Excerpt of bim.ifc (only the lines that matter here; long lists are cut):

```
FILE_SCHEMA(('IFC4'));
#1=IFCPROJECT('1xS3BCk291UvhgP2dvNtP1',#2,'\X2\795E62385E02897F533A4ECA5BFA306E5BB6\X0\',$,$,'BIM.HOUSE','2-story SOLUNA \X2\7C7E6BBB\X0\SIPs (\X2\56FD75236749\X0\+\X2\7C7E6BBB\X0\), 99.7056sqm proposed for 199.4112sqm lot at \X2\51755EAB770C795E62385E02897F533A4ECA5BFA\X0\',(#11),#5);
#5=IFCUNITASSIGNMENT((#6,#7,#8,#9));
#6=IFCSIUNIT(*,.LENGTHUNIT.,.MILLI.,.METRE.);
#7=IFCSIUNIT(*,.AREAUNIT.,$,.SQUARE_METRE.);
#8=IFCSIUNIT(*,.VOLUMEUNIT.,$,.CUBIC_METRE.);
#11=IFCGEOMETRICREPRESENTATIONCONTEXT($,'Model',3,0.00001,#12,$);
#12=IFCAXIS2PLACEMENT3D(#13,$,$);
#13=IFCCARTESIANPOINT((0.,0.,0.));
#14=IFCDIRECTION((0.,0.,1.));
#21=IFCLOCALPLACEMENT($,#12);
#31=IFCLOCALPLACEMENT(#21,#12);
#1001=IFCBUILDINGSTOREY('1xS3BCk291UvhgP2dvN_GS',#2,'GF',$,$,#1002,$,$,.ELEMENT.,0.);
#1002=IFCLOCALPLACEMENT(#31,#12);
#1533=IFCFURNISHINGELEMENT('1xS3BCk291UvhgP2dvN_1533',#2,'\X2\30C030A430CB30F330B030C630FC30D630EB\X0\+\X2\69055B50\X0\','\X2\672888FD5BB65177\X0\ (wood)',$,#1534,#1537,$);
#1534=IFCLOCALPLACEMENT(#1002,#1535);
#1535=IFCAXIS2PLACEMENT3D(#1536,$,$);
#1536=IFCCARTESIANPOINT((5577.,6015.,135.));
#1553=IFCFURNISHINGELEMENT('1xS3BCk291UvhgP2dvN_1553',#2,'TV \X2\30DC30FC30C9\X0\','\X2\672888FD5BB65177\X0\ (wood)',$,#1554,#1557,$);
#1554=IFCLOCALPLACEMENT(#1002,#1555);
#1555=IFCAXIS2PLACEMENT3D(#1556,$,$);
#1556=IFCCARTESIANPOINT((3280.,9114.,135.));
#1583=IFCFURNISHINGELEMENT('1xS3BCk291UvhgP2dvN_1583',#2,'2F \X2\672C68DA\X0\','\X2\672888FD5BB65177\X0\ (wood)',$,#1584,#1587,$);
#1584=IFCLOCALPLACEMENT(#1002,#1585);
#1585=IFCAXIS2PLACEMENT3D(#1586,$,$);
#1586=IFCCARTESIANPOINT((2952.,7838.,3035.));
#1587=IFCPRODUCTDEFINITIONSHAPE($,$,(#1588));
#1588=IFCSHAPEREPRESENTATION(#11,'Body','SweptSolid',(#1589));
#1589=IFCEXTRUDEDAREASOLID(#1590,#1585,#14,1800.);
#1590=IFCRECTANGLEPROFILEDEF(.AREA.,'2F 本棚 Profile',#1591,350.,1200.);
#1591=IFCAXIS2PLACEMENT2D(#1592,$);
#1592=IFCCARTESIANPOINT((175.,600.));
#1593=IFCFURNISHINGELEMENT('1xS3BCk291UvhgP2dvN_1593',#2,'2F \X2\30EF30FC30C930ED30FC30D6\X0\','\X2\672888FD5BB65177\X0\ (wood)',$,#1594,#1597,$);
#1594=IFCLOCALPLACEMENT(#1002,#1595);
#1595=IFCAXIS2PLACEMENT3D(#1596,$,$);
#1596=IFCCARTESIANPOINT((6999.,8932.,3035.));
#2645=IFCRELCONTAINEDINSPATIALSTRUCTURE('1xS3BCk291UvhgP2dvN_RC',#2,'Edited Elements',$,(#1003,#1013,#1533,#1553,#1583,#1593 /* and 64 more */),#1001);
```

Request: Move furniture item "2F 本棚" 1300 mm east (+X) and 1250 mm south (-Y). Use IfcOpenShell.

```python
import ifcopenshell
import ifcopenshell.api.geometry
import ifcopenshell.util.placement
import ifcopenshell.util.unit

model = ifcopenshell.open("bim.ifc")
unit_scale = ifcopenshell.util.unit.calculate_unit_scale(model)

item = model.by_guid("1xS3BCk291UvhgP2dvN_1583")
matrix = ifcopenshell.util.placement.get_local_placement(item.ObjectPlacement)
matrix[0, 3] += 1.3 / unit_scale
matrix[1, 3] -= 1.25 / unit_scale
ifcopenshell.api.geometry.edit_object_placement(model, product=item, matrix=matrix, is_si=False)

print(ifcopenshell.util.placement.get_local_placement(item.ObjectPlacement).round(3) + 0.0)

model.write("bim_v2.ifc")
```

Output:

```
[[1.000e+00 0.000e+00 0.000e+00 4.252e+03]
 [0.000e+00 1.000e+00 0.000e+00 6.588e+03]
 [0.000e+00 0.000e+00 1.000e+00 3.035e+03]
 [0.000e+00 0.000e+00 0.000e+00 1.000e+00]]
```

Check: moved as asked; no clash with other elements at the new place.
